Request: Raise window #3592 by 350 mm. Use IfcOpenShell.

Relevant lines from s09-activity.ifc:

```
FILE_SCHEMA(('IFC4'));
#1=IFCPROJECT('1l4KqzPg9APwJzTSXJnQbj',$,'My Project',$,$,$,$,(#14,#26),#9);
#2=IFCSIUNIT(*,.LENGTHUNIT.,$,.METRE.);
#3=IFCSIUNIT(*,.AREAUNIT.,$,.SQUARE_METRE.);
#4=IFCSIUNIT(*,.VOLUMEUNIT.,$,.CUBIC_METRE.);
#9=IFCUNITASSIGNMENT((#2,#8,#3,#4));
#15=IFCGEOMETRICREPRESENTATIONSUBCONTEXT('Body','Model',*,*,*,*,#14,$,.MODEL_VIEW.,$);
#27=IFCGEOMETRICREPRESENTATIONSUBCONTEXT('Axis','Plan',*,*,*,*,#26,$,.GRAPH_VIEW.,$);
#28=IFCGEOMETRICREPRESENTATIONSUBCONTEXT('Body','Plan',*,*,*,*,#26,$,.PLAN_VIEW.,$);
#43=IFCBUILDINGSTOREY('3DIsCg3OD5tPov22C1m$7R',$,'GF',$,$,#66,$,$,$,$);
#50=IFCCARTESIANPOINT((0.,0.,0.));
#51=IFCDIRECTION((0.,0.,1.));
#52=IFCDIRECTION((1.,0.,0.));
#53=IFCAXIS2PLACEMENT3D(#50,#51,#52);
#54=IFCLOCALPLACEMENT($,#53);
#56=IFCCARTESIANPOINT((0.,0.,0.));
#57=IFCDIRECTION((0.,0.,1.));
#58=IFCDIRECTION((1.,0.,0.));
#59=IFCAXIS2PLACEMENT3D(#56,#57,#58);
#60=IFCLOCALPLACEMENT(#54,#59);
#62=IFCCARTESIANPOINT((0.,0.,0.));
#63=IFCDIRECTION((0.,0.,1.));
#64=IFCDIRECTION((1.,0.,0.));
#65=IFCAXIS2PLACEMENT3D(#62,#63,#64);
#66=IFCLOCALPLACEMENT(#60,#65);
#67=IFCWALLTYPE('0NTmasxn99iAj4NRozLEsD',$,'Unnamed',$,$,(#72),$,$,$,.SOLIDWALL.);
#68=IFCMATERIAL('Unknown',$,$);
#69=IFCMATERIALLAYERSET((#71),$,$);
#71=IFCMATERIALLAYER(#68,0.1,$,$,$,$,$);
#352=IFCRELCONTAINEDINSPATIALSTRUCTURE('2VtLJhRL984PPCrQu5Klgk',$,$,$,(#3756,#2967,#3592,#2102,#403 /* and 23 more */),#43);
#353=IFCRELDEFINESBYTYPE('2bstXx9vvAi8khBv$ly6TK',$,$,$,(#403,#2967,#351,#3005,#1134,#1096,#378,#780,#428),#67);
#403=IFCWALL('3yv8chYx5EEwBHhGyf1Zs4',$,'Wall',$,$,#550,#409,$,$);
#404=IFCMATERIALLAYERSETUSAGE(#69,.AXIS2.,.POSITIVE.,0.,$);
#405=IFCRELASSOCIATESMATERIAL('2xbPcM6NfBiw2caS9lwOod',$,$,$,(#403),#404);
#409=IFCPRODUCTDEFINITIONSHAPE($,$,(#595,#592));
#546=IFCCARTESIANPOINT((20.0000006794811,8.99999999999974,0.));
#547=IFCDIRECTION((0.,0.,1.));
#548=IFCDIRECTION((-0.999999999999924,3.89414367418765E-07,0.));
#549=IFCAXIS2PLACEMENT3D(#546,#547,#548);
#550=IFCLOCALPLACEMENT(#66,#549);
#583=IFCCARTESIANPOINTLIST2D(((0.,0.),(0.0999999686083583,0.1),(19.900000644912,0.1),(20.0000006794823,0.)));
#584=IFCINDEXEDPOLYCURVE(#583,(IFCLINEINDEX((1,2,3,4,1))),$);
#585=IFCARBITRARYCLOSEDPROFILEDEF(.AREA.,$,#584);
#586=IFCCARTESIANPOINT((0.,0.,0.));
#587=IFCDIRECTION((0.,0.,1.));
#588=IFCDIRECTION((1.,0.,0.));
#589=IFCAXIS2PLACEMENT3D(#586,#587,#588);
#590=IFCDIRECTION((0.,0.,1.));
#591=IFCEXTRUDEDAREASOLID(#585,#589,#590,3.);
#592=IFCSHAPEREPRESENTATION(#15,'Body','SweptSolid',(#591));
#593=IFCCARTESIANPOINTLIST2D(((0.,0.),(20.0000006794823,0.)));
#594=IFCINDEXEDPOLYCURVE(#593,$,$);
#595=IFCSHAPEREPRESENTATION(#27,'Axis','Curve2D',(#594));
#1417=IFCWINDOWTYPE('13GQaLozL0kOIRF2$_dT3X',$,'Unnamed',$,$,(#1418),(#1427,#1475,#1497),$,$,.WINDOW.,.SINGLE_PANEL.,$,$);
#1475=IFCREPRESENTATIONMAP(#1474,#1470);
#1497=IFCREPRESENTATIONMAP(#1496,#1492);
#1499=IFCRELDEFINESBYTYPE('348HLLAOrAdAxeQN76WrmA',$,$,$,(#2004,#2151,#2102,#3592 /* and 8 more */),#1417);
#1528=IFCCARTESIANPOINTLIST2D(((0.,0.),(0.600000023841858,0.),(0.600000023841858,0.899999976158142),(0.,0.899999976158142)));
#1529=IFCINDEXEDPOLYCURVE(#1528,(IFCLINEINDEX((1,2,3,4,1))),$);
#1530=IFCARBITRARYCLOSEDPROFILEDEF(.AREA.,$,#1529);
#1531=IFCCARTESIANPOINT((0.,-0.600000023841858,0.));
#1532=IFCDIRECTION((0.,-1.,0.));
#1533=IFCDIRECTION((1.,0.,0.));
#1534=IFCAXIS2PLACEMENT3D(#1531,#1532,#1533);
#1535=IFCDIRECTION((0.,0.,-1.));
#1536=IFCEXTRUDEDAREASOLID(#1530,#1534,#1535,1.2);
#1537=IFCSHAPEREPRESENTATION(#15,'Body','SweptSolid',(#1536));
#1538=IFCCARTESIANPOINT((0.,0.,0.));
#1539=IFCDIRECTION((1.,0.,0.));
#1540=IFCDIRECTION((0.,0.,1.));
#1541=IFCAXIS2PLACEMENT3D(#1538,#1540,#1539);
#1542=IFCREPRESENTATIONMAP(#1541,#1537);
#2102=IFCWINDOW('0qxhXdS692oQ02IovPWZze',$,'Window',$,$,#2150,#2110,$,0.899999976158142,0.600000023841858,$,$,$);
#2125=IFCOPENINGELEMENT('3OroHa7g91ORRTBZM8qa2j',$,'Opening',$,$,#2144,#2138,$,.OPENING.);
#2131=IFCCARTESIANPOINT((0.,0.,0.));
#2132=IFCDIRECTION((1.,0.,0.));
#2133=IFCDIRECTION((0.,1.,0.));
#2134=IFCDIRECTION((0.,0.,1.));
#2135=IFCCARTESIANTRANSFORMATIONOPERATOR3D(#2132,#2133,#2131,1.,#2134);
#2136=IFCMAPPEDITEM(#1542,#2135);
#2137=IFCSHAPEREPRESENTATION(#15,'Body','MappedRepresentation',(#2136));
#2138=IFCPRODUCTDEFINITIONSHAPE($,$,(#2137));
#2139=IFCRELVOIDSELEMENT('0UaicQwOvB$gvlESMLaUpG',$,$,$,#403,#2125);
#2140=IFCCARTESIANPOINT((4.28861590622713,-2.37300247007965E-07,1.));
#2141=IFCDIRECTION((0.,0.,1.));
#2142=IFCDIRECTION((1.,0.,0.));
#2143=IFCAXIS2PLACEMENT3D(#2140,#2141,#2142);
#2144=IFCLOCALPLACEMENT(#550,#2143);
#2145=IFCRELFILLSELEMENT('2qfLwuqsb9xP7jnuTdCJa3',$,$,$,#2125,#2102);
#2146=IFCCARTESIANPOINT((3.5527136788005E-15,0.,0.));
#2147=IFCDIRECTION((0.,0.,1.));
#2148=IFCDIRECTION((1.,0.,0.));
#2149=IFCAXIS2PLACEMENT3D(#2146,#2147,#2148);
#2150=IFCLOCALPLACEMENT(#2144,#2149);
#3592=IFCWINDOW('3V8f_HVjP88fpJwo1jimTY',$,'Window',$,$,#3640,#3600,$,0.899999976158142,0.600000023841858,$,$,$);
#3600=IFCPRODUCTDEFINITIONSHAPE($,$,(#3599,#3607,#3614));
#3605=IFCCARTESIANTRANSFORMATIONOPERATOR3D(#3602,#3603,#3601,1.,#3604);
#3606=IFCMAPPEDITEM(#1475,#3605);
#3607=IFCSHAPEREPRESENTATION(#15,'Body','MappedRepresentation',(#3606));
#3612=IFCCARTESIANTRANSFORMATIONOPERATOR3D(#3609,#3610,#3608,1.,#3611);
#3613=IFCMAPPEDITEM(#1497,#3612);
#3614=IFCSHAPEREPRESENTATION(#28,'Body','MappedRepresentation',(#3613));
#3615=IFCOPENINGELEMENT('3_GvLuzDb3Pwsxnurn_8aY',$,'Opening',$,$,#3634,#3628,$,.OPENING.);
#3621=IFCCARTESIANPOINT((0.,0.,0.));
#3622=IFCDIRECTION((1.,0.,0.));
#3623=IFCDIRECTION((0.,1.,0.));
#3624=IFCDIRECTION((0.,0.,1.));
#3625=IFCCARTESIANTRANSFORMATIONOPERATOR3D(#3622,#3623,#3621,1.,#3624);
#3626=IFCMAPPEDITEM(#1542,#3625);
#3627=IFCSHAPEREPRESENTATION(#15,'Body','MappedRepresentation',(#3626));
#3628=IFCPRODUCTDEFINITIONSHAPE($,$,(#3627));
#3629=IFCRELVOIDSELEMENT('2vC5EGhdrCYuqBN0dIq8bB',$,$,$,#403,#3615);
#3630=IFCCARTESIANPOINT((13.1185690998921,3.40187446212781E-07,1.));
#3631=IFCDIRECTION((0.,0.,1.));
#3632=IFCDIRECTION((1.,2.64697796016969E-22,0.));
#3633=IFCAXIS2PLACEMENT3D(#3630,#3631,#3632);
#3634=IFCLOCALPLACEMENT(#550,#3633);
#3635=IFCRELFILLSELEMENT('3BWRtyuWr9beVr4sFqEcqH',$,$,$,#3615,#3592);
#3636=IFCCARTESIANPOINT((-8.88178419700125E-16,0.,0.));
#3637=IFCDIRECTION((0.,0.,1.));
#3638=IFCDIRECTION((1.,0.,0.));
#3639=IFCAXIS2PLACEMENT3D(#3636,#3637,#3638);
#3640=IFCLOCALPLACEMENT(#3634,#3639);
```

```python
import numpy as np
import ifcopenshell
import ifcopenshell.api.geometry
import ifcopenshell.util.placement
import ifcopenshell.util.unit

model = ifcopenshell.open("s09-activity.ifc")
unit_scale = ifcopenshell.util.unit.calculate_unit_scale(model)

window = model.by_id(3592)
opening = window.FillsVoids[0].RelatingOpeningElement
dz = 0.35 / unit_scale

shift = np.array([0.0, 0.0, dz])
# The window is placed relative to its opening, so it follows when the opening moves.
matrix = ifcopenshell.util.placement.get_local_placement(opening.ObjectPlacement)
matrix[:3, 3] += shift
ifcopenshell.api.geometry.edit_object_placement(
    model, product=opening, matrix=matrix, is_si=False, should_transform_children=True
)

print(f"moved by {dz * unit_scale:+.3f} m")

model.write("s09-activity-out.ifc")
```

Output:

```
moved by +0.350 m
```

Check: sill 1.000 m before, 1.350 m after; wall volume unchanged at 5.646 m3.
